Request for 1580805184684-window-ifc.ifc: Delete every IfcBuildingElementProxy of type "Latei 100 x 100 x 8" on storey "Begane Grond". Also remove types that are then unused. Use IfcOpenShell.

First a look at what the model holds.

```python
import ifcopenshell
import ifcopenshell.util.element

model = ifcopenshell.open("1580805184684-window-ifc.ifc")
print(model.schema)
storey = next(s for s in model.by_type("IfcBuildingStorey") if s.Name == "Begane Grond")
proxies = [e for e in ifcopenshell.util.element.get_decomposition(storey) if e.is_a("IfcBuildingElementProxy")]
seen = {}
for e in proxies:
    element_type = ifcopenshell.util.element.get_type(e)
    name = element_type.Name if element_type not in (None, e) else None
    seen[name] = seen.get(name, 0) + 1
for name, count in sorted(seen.items(), key=str):
    print(count, "x", name)
```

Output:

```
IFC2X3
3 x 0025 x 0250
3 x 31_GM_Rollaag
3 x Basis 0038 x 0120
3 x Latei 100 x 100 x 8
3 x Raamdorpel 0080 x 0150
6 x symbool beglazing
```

```python
import ifcopenshell
import ifcopenshell.api.root
import ifcopenshell.util.element

model = ifcopenshell.open("1580805184684-window-ifc.ifc")

storey = next(s for s in model.by_type("IfcBuildingStorey") if s.Name == "Begane Grond")
proxies = [e for e in ifcopenshell.util.element.get_decomposition(storey) if e.is_a("IfcBuildingElementProxy")]
targets = [e for e in proxies if (t := ifcopenshell.util.element.get_type(e)) not in (None, e) and t.Name == "Latei 100 x 100 x 8"]
types = {ifcopenshell.util.element.get_type(e) for e in targets} - {None, *targets}

for e in targets:
    ifcopenshell.api.root.remove_product(model, product=e)
print(len(targets), "removed")

unused = [t for t in types if not ifcopenshell.util.element.get_types(t)]
for t in unused:
    ifcopenshell.api.root.remove_product(model, product=t)
print(len(unused), "unused types removed")

model.write("1580805184684-window-ifc_edited.ifc")
```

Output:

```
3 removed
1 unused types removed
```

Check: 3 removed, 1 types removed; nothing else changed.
